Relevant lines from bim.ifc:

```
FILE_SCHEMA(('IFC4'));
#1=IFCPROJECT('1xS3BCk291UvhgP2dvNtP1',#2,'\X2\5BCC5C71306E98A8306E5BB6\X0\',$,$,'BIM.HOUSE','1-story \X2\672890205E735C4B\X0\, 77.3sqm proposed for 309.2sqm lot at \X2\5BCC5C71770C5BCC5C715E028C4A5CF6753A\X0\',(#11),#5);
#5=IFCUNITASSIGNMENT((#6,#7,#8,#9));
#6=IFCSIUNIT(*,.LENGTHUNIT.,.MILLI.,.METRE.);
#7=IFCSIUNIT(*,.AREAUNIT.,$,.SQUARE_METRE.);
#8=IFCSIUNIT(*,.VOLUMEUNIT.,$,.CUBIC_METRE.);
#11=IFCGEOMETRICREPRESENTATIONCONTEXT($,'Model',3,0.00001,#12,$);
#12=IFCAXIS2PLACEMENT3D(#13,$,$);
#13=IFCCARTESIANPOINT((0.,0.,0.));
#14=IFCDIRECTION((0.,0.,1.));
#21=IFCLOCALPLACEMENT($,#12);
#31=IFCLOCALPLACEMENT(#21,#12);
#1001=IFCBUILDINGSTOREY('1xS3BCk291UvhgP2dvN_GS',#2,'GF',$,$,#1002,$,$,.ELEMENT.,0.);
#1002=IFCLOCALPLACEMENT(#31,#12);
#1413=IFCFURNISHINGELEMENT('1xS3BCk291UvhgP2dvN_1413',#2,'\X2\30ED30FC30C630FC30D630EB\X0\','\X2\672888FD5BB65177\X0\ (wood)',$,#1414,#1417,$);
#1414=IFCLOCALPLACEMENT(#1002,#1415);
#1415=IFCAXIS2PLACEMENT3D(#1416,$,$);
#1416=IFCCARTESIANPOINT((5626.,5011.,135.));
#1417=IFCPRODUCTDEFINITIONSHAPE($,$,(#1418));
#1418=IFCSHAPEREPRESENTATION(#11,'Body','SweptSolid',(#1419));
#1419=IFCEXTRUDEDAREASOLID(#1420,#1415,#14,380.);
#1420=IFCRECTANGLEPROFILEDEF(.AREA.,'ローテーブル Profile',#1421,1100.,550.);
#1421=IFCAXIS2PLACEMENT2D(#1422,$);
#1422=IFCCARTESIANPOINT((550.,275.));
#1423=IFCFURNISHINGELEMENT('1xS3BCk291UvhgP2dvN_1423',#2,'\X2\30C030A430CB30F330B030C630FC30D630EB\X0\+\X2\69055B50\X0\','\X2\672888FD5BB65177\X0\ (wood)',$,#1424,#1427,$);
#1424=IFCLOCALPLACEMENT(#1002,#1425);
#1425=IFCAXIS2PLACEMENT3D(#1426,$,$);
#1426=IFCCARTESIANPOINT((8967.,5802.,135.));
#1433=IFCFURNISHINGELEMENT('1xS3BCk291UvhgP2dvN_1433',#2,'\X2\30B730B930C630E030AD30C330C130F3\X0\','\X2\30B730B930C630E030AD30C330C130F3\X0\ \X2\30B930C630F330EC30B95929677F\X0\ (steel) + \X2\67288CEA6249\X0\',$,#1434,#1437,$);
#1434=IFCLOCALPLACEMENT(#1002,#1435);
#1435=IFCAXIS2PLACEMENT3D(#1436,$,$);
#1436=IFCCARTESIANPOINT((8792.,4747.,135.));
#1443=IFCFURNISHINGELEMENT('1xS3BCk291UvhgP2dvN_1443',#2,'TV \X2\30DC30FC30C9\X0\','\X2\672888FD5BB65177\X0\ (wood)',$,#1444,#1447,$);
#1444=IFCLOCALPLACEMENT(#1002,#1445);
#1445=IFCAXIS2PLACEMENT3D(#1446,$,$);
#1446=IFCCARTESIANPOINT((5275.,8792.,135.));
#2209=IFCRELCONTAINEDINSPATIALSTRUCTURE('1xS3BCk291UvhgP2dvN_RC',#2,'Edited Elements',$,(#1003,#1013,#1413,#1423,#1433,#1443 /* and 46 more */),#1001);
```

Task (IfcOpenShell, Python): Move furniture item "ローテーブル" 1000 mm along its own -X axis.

```python
import ifcopenshell
import ifcopenshell.api.geometry
import ifcopenshell.util.placement

model = ifcopenshell.open("bim.ifc")

item = model.by_guid("1xS3BCk291UvhgP2dvN_1413")
matrix = ifcopenshell.util.placement.get_local_placement(item.ObjectPlacement)
matrix[:3, 3] -= matrix[:3, 0] * 1000.0
ifcopenshell.api.geometry.edit_object_placement(model, product=item, matrix=matrix, is_si=False)

print(ifcopenshell.util.placement.get_local_placement(item.ObjectPlacement).round(3) + 0.0)

model.write("bim_v2.ifc")
```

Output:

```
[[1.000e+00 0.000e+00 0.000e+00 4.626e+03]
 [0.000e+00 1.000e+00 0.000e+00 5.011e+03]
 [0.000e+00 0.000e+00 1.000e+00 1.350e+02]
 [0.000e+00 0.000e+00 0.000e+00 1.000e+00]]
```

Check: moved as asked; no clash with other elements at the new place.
